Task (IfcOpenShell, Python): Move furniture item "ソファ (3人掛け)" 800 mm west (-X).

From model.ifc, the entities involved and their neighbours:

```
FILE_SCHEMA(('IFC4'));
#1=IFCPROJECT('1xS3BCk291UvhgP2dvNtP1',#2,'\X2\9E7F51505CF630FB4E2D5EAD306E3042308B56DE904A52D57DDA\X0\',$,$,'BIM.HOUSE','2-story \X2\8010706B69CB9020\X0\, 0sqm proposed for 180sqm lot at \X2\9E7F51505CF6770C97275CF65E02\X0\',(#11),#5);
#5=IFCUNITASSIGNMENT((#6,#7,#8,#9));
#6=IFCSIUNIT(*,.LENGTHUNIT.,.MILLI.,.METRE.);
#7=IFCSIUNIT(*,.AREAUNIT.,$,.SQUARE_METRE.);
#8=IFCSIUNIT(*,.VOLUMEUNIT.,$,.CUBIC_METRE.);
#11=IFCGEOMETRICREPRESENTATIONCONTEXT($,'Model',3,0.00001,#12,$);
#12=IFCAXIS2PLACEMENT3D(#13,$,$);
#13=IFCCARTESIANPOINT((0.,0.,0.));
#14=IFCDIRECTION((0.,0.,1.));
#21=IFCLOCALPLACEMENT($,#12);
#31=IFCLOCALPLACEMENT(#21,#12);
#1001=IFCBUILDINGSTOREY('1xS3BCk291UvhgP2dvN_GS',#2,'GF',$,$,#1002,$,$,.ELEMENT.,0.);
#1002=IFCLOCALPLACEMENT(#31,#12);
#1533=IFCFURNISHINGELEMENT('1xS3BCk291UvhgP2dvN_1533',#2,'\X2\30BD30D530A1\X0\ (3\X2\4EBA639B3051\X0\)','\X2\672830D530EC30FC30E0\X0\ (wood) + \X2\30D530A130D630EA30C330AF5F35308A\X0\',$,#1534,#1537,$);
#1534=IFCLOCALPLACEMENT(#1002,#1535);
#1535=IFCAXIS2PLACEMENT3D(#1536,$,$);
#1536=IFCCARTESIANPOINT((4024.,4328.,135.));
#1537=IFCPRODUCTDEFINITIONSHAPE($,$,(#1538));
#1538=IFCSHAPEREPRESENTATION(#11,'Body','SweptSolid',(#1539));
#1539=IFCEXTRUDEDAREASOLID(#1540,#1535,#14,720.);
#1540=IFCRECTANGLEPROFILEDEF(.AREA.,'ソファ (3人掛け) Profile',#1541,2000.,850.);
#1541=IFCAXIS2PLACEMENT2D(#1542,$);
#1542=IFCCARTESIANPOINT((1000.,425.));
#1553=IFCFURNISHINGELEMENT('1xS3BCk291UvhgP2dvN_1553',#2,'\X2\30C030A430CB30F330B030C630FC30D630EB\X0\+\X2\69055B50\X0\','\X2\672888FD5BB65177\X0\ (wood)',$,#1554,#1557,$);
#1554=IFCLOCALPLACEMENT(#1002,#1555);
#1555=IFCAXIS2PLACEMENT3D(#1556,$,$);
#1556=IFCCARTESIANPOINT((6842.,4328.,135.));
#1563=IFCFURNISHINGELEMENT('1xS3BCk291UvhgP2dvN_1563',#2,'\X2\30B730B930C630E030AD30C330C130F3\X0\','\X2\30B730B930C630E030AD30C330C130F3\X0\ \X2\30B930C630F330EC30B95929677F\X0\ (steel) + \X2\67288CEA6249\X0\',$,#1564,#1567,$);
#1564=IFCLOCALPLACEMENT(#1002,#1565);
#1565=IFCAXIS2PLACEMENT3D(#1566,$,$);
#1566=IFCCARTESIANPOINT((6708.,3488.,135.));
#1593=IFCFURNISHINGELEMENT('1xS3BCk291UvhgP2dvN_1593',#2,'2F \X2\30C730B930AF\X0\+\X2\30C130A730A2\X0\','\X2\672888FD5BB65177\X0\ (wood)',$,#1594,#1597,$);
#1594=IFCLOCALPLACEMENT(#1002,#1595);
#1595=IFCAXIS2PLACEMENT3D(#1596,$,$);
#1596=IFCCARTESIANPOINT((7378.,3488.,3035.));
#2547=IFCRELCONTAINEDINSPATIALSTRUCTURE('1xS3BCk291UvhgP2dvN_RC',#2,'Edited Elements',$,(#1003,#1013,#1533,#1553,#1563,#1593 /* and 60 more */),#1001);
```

```python
import ifcopenshell
import ifcopenshell.api.geometry
import ifcopenshell.util.placement

model = ifcopenshell.open("model.ifc")

item = model.by_guid("1xS3BCk291UvhgP2dvN_1533")
matrix = ifcopenshell.util.placement.get_local_placement(item.ObjectPlacement)
matrix[0, 3] -= 800.0
ifcopenshell.api.geometry.edit_object_placement(model, product=item, matrix=matrix, is_si=False)

print(ifcopenshell.util.placement.get_local_placement(item.ObjectPlacement).round(3) + 0.0)

model.write("model_v2.ifc")
```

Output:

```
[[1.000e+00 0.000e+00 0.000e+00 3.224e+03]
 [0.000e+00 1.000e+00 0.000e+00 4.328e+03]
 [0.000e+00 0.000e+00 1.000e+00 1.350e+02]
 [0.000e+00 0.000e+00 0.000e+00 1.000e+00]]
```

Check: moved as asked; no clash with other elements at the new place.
